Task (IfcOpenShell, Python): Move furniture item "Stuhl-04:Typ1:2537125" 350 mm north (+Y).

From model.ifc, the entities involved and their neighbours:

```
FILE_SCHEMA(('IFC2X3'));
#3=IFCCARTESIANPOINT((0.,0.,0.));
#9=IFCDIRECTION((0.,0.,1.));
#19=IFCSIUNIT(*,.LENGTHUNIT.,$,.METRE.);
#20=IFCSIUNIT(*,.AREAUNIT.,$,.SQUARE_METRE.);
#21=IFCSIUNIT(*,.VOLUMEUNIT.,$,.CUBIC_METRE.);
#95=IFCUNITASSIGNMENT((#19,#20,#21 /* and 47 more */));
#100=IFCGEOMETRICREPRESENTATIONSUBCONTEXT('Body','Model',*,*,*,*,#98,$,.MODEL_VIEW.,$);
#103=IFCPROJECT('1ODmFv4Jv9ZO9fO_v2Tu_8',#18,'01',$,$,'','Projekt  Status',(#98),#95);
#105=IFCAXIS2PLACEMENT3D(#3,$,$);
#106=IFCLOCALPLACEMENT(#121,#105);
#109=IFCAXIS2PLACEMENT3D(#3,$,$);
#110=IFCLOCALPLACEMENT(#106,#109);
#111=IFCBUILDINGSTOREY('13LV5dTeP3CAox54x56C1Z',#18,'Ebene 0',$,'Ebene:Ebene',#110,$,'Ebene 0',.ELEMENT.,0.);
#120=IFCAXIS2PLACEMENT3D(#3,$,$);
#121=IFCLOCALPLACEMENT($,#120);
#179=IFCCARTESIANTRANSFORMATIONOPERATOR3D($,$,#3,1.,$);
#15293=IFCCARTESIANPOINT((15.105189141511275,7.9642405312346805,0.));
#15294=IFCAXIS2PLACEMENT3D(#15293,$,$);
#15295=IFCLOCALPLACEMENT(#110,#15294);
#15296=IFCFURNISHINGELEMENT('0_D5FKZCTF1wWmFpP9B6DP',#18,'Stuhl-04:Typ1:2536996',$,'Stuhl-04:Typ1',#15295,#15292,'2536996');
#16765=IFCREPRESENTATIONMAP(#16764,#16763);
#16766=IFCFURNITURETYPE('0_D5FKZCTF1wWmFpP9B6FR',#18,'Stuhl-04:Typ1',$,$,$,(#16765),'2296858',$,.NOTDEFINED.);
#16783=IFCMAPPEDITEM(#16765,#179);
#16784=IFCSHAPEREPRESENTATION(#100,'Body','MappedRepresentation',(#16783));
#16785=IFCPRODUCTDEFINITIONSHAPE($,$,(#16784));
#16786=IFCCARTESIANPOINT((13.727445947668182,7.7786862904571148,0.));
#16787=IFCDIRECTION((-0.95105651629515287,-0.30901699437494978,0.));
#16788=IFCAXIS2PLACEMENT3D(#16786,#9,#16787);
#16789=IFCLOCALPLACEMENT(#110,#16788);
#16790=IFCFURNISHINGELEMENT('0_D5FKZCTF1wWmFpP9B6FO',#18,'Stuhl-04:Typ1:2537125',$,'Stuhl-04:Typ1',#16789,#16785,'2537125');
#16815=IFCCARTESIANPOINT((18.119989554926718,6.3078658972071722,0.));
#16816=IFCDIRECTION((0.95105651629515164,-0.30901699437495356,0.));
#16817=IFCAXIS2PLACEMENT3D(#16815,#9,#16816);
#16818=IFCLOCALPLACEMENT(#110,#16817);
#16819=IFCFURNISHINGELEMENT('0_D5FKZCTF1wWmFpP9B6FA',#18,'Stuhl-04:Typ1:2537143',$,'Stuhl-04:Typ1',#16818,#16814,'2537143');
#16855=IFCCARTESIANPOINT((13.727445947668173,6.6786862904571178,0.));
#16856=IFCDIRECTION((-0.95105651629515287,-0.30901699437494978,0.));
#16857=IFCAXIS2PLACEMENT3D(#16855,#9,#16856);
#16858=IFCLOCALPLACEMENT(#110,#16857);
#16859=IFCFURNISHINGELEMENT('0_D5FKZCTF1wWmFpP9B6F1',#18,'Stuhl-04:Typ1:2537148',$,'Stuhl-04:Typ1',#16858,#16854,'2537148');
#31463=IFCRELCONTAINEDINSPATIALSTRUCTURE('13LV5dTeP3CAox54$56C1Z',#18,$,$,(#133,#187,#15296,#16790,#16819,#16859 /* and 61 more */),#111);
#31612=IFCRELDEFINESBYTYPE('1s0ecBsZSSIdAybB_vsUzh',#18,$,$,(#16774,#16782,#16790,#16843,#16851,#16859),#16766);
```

```python
import ifcopenshell
import ifcopenshell.api.geometry
import ifcopenshell.util.placement
import ifcopenshell.util.unit

model = ifcopenshell.open("model.ifc")
unit_scale = ifcopenshell.util.unit.calculate_unit_scale(model)

item = model.by_id(16790)
matrix = ifcopenshell.util.placement.get_local_placement(item.ObjectPlacement)
matrix[1, 3] += 0.35 / unit_scale
ifcopenshell.api.geometry.edit_object_placement(model, product=item, matrix=matrix, is_si=False)

print(ifcopenshell.util.placement.get_local_placement(item.ObjectPlacement).round(3) + 0.0)

model.write("model_updated.ifc")
```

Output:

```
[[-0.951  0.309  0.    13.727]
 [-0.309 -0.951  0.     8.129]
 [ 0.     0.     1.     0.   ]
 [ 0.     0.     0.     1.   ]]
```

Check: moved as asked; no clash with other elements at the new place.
